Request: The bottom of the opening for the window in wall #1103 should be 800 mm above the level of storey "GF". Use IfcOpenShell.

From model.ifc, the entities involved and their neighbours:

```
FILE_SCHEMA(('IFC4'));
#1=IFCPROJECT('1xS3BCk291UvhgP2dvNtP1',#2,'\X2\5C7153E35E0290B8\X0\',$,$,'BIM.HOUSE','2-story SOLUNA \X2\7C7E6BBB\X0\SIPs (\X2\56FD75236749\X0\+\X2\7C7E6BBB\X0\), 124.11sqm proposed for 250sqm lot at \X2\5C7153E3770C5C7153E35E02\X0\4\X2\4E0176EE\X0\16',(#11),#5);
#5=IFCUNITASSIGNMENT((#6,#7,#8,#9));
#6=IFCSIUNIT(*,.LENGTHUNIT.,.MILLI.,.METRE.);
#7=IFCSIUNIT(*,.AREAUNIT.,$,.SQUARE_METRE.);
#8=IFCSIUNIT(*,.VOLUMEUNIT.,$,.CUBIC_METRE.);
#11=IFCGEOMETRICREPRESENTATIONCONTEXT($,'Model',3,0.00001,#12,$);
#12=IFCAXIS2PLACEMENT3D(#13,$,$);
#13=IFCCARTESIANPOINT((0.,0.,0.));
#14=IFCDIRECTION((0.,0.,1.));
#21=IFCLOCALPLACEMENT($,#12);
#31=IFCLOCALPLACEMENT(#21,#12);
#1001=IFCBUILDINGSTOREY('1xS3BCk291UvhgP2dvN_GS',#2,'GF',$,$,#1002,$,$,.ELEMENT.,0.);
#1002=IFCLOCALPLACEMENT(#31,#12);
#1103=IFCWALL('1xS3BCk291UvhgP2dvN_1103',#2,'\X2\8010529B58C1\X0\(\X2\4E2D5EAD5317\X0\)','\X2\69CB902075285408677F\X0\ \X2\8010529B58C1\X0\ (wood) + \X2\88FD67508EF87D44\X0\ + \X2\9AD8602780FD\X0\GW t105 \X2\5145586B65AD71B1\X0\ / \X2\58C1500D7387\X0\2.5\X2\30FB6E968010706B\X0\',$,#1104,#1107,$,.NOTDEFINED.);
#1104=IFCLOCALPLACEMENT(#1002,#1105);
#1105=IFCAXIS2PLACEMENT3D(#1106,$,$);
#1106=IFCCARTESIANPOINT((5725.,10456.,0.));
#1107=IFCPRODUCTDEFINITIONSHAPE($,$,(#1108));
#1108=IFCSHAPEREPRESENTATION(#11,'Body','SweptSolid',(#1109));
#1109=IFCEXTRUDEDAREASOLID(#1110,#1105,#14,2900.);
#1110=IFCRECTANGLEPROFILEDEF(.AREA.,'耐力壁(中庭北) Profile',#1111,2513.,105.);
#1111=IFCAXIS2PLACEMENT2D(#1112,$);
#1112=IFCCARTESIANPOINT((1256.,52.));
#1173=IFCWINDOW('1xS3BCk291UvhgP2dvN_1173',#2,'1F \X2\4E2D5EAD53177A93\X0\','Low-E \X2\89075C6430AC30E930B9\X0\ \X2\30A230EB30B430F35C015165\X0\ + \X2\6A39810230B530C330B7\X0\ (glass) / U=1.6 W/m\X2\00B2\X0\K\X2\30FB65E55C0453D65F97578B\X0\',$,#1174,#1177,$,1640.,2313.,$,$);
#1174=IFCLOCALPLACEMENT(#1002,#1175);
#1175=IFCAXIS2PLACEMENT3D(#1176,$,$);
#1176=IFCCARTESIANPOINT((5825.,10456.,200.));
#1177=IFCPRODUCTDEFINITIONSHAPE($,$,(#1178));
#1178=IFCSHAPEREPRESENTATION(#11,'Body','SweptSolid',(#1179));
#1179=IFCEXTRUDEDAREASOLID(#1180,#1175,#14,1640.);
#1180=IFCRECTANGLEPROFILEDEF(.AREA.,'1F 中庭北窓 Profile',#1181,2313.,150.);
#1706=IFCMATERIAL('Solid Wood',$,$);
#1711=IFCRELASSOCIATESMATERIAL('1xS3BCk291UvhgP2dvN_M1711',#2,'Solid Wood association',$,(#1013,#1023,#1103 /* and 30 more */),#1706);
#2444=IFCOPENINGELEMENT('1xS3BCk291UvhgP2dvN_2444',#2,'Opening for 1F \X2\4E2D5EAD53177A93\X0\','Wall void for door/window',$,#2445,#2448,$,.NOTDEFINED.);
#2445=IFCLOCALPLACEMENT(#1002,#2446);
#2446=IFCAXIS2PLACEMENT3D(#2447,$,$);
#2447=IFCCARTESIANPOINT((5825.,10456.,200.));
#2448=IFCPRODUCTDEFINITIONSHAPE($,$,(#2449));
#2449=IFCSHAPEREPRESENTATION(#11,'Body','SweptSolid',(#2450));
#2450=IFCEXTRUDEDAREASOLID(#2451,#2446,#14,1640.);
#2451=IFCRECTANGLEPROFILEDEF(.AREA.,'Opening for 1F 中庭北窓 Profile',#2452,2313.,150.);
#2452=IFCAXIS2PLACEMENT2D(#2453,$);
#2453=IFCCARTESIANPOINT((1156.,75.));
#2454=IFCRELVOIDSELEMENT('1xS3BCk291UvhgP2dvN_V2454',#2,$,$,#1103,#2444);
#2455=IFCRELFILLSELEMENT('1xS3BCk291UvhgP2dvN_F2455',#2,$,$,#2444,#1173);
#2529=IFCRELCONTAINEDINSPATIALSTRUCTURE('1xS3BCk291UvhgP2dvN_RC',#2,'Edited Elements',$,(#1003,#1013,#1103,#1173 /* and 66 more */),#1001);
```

```python
import numpy as np
import ifcopenshell
import ifcopenshell.api.geometry
import ifcopenshell.geom
import ifcopenshell.util.element
import ifcopenshell.util.placement
import ifcopenshell.util.shape
import ifcopenshell.util.unit

model = ifcopenshell.open("model.ifc")
unit_scale = ifcopenshell.util.unit.calculate_unit_scale(model)

window = model.by_guid("1xS3BCk291UvhgP2dvN_1173")
opening = window.FillsVoids[0].RelatingOpeningElement
storey = ifcopenshell.util.element.get_container(window, ifc_class="IfcBuildingStorey")
level = ifcopenshell.util.placement.get_local_placement(storey.ObjectPlacement)[2, 3]

# The opening's origin need not be at the sill, so measure its lowest point.
shape = ifcopenshell.geom.create_shape(ifcopenshell.geom.settings(), opening)
bottom = ifcopenshell.util.shape.get_shape_bottom_elevation(shape, shape.geometry) / unit_scale
dz = level + 800.0 - bottom

shift = np.array([0.0, 0.0, dz])
# The window is not placed relative to its opening, so move both.
for product in (opening, window):
    matrix = ifcopenshell.util.placement.get_local_placement(product.ObjectPlacement)
    matrix[:3, 3] += shift
    ifcopenshell.api.geometry.edit_object_placement(model, product=product, matrix=matrix, is_si=False)

print(f"moved by {dz * unit_scale:+.3f} m")

model.write("model_rev.ifc")
```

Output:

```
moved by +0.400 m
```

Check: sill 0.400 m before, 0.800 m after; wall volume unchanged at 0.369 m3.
